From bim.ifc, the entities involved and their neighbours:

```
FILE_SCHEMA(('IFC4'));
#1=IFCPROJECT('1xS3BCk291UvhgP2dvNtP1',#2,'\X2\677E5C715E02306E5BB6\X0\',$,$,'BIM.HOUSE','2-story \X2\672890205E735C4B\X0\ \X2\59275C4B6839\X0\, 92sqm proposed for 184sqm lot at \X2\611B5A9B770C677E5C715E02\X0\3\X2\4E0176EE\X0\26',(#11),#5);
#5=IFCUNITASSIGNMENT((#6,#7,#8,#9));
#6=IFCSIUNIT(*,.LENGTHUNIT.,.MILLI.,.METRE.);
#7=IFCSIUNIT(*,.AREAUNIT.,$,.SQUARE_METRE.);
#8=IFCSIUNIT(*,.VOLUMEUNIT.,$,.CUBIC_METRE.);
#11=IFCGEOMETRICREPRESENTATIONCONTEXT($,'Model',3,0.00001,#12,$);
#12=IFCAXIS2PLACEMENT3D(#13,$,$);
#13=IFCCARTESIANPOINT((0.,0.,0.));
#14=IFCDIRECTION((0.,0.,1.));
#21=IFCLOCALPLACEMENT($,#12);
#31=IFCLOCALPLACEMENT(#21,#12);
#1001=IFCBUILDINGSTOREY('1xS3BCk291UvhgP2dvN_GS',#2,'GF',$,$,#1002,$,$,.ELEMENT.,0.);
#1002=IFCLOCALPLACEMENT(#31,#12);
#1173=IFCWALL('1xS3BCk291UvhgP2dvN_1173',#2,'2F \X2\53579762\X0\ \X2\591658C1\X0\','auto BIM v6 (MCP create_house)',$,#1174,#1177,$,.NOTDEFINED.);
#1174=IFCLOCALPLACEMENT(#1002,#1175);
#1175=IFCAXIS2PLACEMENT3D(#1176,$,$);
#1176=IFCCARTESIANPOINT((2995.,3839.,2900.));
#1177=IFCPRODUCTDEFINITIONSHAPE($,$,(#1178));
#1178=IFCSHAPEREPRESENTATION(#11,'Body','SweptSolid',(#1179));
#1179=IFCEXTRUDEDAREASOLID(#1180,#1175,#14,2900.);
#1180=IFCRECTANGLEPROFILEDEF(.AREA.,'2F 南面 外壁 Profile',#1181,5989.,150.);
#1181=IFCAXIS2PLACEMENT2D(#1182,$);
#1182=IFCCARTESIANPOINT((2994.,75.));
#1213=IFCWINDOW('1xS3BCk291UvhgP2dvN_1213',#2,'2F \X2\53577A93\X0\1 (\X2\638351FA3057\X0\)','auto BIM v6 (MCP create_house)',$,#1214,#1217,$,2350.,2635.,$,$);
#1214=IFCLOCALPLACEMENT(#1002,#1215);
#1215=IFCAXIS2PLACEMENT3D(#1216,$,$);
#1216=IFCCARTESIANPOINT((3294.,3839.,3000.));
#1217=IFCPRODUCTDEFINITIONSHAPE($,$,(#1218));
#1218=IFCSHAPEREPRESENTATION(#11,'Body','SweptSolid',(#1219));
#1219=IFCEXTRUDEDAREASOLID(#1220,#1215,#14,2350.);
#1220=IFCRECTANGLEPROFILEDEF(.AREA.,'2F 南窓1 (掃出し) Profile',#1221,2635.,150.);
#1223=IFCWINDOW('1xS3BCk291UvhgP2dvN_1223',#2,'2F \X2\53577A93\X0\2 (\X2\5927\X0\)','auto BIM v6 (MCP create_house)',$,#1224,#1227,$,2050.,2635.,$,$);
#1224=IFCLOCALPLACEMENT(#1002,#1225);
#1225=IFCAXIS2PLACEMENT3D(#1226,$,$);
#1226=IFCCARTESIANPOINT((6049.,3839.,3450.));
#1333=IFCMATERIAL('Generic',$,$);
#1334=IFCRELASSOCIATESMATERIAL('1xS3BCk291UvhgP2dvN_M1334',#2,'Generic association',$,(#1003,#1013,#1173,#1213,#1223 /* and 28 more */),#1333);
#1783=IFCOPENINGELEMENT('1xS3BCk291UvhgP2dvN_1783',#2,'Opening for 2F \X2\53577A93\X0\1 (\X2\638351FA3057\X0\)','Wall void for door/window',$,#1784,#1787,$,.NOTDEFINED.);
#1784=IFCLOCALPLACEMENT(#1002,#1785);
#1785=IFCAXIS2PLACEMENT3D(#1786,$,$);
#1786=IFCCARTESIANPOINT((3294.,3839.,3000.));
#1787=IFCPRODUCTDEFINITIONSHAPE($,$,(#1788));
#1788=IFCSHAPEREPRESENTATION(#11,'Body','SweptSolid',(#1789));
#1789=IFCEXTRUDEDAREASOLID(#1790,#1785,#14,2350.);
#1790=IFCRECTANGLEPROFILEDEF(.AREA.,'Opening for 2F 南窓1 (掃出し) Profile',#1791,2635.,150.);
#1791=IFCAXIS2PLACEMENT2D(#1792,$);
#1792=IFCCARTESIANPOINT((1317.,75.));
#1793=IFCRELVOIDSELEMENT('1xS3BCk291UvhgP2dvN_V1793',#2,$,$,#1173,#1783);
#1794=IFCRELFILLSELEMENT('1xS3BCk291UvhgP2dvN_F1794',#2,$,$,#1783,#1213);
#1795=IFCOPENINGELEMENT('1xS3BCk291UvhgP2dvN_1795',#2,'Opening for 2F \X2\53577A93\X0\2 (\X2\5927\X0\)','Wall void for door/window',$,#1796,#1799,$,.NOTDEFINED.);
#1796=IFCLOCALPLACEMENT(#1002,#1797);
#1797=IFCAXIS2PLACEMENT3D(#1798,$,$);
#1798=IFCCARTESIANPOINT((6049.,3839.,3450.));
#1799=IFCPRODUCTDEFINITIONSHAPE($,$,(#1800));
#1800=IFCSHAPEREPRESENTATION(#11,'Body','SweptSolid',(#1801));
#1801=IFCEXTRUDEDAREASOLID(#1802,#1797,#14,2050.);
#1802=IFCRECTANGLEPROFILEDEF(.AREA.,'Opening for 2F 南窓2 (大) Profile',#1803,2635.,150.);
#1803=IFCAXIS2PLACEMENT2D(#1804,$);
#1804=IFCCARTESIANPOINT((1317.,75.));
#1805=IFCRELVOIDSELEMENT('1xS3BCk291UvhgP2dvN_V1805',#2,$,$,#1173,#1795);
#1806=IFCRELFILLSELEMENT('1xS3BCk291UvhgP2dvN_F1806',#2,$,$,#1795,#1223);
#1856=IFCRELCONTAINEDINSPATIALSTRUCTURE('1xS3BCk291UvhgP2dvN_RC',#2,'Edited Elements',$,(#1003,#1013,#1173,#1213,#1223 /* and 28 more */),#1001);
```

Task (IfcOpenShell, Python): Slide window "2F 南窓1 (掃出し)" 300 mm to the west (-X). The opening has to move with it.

```python
import ifcopenshell
import ifcopenshell.api.geometry
import ifcopenshell.util.placement
import ifcopenshell.util.unit

model = ifcopenshell.open("bim.ifc")
unit_scale = ifcopenshell.util.unit.calculate_unit_scale(model)

window = model.by_id(1213)
opening = window.FillsVoids[0].RelatingOpeningElement
wall = opening.VoidsElements[0].RelatingBuildingElement

wall_matrix = ifcopenshell.util.placement.get_local_placement(wall.ObjectPlacement)
shift = wall_matrix[:3, 0] * -0.3 / unit_scale
before = ifcopenshell.util.placement.get_local_placement(window.ObjectPlacement)[:3, 3].copy()

# The window is not placed relative to its opening, so move both.
for product in (opening, window):
    matrix = ifcopenshell.util.placement.get_local_placement(product.ObjectPlacement)
    matrix[:3, 3] += shift
    ifcopenshell.api.geometry.edit_object_placement(model, product=product, matrix=matrix, is_si=False)

after = ifcopenshell.util.placement.get_local_placement(window.ObjectPlacement)[:3, 3]
print("window moved by", (after - before).round(3) + 0.0)

model.write("bim_v2.ifc")
```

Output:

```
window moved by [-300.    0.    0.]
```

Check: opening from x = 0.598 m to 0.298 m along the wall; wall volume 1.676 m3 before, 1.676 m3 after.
